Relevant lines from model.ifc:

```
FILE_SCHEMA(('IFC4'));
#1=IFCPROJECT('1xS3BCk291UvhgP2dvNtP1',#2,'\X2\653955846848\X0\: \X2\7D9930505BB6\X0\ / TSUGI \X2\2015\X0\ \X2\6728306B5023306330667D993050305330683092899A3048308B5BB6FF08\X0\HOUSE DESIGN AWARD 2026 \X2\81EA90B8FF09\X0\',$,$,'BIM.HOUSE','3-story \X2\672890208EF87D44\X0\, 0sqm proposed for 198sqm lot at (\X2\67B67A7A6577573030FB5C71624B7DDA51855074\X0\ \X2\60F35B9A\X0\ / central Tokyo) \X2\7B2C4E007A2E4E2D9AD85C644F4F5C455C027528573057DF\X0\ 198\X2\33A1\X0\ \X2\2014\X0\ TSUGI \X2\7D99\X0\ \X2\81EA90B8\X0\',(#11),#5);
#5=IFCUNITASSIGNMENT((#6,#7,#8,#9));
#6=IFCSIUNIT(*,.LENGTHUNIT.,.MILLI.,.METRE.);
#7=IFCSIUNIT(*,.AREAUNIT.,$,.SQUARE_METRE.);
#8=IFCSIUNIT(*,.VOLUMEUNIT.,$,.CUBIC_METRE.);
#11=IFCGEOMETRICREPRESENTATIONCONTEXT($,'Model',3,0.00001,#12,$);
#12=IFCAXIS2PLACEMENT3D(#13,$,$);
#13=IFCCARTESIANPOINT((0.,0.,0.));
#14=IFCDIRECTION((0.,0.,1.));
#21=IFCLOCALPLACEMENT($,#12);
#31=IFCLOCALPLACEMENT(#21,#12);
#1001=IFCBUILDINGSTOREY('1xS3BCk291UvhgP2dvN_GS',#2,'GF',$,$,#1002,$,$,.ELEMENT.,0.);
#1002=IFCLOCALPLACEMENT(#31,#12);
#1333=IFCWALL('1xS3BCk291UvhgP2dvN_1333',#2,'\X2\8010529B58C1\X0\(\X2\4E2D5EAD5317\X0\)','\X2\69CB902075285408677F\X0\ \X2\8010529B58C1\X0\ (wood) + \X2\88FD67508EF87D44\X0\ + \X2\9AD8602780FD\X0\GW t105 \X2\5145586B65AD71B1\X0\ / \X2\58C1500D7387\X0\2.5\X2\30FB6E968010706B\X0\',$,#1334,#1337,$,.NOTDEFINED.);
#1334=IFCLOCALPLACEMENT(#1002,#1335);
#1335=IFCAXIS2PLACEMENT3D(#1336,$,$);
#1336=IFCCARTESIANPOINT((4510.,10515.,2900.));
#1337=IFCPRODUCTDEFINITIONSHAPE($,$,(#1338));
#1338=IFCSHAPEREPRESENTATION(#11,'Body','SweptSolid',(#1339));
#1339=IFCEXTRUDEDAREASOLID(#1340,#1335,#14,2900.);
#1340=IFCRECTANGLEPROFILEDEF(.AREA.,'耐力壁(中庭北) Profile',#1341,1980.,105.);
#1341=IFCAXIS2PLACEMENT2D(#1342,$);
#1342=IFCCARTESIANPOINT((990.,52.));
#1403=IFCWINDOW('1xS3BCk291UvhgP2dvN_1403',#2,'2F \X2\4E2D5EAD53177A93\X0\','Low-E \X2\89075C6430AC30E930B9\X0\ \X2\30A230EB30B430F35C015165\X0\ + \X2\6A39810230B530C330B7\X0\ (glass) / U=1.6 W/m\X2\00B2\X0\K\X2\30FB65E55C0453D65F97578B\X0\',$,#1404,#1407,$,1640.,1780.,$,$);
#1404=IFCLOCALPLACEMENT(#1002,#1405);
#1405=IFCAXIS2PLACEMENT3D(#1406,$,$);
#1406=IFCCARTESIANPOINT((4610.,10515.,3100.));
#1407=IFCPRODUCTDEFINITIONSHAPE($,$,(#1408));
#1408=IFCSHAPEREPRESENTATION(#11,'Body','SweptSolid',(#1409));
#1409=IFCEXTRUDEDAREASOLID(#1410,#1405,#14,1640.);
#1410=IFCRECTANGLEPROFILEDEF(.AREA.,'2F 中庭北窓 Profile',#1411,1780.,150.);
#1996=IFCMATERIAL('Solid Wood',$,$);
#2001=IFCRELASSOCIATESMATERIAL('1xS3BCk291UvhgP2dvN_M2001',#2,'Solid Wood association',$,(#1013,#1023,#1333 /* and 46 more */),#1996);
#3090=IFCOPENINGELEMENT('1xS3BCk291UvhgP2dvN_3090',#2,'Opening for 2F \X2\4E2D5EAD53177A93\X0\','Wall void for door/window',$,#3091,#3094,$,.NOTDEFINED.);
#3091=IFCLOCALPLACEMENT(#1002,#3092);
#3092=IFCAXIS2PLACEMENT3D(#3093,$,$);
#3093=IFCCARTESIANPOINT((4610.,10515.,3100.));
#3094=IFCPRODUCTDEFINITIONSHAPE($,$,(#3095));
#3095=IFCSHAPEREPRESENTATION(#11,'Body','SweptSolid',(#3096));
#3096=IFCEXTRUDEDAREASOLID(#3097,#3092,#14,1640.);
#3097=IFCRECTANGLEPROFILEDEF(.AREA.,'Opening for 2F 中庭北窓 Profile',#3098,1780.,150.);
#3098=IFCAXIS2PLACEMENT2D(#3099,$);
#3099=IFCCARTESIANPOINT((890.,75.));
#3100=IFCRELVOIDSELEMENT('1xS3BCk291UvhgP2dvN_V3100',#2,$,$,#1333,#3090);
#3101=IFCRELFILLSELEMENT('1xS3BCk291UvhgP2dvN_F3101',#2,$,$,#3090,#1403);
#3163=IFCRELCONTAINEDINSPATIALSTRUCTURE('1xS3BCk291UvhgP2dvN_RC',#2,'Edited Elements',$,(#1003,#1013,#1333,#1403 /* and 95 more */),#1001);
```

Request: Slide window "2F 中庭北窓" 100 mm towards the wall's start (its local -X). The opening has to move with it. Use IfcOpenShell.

```python
import ifcopenshell
import ifcopenshell.api.geometry
import ifcopenshell.util.placement
import ifcopenshell.util.unit

model = ifcopenshell.open("model.ifc")
unit_scale = ifcopenshell.util.unit.calculate_unit_scale(model)

window = model.by_id(1403)
opening = window.FillsVoids[0].RelatingOpeningElement
wall = opening.VoidsElements[0].RelatingBuildingElement

wall_matrix = ifcopenshell.util.placement.get_local_placement(wall.ObjectPlacement)
shift = wall_matrix[:3, 0] * -0.1 / unit_scale
before = ifcopenshell.util.placement.get_local_placement(window.ObjectPlacement)[:3, 3].copy()

# The window is not placed relative to its opening, so move both.
for product in (opening, window):
    matrix = ifcopenshell.util.placement.get_local_placement(product.ObjectPlacement)
    matrix[:3, 3] += shift
    ifcopenshell.api.geometry.edit_object_placement(model, product=product, matrix=matrix, is_si=False)

after = ifcopenshell.util.placement.get_local_placement(window.ObjectPlacement)[:3, 3]
print("window moved by", (after - before).round(3) + 0.0)

model.write("model_edited.ifc")
```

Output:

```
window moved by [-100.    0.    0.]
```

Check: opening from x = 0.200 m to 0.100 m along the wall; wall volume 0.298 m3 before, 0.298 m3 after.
